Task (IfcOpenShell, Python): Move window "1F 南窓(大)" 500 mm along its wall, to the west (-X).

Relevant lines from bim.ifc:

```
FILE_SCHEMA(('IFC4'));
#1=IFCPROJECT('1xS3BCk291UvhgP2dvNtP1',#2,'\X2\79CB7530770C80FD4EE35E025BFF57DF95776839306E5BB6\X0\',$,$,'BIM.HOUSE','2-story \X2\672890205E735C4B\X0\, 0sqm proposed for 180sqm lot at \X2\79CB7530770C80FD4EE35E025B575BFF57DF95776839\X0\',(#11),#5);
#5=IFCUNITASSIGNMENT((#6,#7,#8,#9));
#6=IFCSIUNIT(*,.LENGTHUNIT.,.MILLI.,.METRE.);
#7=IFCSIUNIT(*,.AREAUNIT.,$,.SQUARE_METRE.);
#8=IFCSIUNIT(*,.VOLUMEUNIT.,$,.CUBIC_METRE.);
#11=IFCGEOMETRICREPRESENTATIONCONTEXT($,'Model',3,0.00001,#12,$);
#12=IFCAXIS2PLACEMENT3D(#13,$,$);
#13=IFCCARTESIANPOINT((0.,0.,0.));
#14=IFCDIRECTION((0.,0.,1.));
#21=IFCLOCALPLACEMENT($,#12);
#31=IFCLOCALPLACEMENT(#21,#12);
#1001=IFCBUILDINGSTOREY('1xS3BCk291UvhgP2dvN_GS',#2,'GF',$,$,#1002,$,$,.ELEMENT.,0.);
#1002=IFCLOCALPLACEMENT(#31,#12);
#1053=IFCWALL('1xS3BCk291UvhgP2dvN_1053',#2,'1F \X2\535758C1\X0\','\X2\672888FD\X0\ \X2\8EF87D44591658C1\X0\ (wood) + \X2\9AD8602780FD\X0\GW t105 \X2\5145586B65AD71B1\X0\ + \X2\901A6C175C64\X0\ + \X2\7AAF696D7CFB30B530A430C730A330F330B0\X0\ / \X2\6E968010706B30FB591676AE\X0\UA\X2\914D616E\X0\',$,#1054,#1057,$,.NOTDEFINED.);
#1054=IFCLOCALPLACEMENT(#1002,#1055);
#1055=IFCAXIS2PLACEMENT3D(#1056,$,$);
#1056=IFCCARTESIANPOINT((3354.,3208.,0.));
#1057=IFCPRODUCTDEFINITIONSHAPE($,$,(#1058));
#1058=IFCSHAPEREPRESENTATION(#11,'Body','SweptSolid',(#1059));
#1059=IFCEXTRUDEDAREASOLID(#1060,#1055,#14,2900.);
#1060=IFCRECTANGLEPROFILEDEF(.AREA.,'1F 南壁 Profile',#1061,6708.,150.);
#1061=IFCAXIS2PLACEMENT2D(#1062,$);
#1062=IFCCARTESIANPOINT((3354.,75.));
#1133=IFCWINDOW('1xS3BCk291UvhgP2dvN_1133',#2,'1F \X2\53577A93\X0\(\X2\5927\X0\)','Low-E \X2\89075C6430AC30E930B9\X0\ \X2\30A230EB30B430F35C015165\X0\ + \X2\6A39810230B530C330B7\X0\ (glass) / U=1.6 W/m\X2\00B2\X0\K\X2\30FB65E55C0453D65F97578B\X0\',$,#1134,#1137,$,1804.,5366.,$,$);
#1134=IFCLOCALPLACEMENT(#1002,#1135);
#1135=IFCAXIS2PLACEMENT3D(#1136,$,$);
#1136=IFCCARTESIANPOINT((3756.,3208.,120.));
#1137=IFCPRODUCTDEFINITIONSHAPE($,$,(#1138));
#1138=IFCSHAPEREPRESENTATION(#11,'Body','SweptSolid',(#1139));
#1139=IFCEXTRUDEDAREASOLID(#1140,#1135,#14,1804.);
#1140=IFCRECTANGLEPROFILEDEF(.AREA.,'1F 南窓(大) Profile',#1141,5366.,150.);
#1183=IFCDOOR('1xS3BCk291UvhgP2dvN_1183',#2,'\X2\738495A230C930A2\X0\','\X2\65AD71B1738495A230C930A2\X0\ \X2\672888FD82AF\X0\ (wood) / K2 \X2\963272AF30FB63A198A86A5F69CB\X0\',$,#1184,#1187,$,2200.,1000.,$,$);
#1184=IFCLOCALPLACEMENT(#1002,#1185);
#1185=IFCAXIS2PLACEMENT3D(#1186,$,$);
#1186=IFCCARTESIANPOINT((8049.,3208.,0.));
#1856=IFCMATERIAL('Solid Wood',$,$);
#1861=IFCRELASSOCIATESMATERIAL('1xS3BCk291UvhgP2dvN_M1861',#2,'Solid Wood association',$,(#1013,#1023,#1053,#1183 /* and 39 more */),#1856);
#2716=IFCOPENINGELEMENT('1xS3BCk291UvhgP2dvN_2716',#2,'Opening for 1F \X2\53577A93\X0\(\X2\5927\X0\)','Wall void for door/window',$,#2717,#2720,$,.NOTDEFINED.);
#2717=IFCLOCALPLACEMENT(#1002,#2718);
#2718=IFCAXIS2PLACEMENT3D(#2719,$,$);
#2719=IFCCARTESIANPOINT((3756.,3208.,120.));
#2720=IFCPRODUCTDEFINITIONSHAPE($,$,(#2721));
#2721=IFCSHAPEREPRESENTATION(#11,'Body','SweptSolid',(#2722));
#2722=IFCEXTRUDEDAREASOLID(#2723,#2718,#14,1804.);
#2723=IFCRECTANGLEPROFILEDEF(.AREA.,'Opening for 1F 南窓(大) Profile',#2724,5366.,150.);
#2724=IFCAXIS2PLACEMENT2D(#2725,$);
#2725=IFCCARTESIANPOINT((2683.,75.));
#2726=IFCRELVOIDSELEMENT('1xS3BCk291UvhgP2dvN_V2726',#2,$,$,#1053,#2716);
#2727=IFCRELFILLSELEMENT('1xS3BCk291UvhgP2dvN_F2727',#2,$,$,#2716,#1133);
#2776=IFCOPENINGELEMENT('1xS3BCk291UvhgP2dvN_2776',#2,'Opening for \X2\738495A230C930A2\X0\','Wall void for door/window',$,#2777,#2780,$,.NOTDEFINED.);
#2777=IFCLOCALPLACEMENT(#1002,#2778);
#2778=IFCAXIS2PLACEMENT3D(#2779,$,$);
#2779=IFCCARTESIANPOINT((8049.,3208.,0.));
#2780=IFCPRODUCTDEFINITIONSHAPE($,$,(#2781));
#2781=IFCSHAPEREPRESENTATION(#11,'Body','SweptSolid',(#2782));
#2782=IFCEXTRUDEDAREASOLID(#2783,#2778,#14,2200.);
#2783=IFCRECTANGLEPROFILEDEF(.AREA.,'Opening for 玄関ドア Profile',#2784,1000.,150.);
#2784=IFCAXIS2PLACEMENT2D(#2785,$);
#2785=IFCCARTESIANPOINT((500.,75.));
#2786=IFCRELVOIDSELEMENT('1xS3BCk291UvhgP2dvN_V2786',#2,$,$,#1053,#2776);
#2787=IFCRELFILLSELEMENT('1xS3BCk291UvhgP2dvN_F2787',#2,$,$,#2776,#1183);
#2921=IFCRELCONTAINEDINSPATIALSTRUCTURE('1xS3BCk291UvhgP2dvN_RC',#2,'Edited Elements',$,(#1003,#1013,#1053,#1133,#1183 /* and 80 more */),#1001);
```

```python
import ifcopenshell
import ifcopenshell.api.geometry
import ifcopenshell.util.placement

model = ifcopenshell.open("bim.ifc")

window = model.by_id(1133)
opening = window.FillsVoids[0].RelatingOpeningElement
wall = opening.VoidsElements[0].RelatingBuildingElement

wall_matrix = ifcopenshell.util.placement.get_local_placement(wall.ObjectPlacement)
shift = wall_matrix[:3, 0] * -500.0
before = ifcopenshell.util.placement.get_local_placement(window.ObjectPlacement)[:3, 3].copy()

# The window is not placed relative to its opening, so move both.
for product in (opening, window):
    matrix = ifcopenshell.util.placement.get_local_placement(product.ObjectPlacement)
    matrix[:3, 3] += shift
    ifcopenshell.api.geometry.edit_object_placement(model, product=product, matrix=matrix, is_si=False)

after = ifcopenshell.util.placement.get_local_placement(window.ObjectPlacement)[:3, 3]
print("window moved by", (after - before).round(3) + 0.0)

model.write("bim_updated.ifc")
```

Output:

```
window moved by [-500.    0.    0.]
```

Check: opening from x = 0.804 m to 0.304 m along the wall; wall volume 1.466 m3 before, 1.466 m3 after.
